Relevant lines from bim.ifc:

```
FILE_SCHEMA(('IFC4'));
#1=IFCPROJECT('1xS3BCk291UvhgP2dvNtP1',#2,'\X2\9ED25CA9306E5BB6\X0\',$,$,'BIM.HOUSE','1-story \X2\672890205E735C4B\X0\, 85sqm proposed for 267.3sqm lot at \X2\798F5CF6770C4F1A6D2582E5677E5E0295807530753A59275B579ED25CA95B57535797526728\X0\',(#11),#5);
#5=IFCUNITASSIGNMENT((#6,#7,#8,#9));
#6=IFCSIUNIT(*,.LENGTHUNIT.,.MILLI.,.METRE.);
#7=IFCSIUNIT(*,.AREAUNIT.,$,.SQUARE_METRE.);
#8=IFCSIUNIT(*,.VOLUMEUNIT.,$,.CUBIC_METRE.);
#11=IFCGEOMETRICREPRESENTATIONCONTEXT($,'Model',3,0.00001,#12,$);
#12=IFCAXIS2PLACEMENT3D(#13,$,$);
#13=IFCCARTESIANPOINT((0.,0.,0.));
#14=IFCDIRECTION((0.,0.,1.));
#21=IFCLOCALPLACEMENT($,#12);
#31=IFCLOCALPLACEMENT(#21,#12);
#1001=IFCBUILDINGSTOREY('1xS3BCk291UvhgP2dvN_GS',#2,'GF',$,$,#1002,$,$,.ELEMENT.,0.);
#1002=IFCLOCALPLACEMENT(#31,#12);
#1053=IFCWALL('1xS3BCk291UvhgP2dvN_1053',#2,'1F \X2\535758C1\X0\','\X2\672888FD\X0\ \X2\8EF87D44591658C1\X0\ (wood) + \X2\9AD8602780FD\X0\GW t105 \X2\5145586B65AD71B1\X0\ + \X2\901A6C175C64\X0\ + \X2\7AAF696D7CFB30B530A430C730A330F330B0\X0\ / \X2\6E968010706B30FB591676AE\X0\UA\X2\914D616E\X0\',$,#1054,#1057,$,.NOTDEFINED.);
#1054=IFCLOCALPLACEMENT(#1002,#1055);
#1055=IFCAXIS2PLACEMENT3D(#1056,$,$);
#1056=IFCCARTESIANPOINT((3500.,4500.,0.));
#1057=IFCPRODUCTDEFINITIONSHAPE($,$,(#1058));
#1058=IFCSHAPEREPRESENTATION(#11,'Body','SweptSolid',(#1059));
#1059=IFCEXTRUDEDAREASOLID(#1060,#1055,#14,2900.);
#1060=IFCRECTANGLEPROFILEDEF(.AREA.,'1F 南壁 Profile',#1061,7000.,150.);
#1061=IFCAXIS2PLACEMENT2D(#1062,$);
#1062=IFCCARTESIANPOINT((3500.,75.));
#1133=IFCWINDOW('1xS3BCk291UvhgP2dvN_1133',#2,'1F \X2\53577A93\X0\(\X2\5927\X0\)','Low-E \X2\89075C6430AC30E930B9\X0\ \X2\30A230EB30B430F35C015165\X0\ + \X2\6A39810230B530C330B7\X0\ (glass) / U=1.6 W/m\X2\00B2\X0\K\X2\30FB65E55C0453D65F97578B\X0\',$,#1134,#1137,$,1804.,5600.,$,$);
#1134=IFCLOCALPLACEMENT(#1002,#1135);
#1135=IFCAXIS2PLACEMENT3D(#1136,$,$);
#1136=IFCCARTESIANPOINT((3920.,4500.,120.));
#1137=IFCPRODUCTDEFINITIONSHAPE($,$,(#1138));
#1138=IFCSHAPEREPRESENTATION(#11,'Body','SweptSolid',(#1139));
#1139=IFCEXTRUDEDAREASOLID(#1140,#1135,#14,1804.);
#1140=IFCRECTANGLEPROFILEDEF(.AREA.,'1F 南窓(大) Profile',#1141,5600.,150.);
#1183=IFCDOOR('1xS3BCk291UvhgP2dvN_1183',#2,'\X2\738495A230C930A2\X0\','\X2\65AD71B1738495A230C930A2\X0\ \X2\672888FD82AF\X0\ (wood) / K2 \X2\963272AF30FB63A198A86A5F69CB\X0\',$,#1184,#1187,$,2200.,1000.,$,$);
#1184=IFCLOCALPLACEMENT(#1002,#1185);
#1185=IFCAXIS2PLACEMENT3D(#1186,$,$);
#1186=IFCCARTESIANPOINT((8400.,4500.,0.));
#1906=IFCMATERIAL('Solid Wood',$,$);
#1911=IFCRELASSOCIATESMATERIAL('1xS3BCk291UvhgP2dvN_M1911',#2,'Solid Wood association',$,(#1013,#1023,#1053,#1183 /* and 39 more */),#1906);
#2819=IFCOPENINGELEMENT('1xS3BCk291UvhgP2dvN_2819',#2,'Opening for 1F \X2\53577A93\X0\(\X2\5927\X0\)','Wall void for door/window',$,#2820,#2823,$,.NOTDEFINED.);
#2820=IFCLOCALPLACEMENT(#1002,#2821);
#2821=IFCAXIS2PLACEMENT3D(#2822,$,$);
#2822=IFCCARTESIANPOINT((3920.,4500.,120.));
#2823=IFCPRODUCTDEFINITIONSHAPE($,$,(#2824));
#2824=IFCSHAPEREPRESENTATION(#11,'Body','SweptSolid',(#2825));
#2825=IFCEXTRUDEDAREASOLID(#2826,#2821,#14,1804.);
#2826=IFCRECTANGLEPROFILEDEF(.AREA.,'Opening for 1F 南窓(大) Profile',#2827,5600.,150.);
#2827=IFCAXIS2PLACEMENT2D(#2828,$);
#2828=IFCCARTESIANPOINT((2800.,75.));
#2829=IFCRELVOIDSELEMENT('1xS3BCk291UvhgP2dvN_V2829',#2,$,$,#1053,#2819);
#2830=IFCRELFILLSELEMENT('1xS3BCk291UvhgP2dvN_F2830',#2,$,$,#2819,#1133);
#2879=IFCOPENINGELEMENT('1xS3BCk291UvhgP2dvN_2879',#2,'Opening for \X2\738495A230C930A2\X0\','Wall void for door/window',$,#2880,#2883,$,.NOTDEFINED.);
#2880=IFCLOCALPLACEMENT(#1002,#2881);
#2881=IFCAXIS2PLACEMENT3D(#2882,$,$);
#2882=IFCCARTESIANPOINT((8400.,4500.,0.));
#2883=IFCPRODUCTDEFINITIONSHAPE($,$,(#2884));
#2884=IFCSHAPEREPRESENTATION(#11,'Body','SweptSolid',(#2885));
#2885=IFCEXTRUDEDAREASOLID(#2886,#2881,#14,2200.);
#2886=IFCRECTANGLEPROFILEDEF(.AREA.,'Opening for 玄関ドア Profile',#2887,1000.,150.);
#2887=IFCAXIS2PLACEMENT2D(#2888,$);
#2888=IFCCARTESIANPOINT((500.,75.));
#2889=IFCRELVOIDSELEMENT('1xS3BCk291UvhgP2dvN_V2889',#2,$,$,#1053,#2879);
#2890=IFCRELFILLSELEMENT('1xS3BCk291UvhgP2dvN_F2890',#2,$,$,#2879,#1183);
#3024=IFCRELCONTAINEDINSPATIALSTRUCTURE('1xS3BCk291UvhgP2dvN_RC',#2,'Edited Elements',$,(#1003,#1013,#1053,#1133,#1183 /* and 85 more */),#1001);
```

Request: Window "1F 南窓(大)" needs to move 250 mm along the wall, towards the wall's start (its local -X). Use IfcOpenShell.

```python
import ifcopenshell
import ifcopenshell.api.geometry
import ifcopenshell.util.placement

model = ifcopenshell.open("bim.ifc")

window = model.by_id(1133)
opening = window.FillsVoids[0].RelatingOpeningElement
wall = opening.VoidsElements[0].RelatingBuildingElement

wall_matrix = ifcopenshell.util.placement.get_local_placement(wall.ObjectPlacement)
shift = wall_matrix[:3, 0] * -250.0
before = ifcopenshell.util.placement.get_local_placement(window.ObjectPlacement)[:3, 3].copy()

# The window is not placed relative to its opening, so move both.
for product in (opening, window):
    matrix = ifcopenshell.util.placement.get_local_placement(product.ObjectPlacement)
    matrix[:3, 3] += shift
    ifcopenshell.api.geometry.edit_object_placement(model, product=product, matrix=matrix, is_si=False)

after = ifcopenshell.util.placement.get_local_placement(window.ObjectPlacement)[:3, 3]
print("window moved by", (after - before).round(3) + 0.0)

model.write("bim_v2.ifc")
```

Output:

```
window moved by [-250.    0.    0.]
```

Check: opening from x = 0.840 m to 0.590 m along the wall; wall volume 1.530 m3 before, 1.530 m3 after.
